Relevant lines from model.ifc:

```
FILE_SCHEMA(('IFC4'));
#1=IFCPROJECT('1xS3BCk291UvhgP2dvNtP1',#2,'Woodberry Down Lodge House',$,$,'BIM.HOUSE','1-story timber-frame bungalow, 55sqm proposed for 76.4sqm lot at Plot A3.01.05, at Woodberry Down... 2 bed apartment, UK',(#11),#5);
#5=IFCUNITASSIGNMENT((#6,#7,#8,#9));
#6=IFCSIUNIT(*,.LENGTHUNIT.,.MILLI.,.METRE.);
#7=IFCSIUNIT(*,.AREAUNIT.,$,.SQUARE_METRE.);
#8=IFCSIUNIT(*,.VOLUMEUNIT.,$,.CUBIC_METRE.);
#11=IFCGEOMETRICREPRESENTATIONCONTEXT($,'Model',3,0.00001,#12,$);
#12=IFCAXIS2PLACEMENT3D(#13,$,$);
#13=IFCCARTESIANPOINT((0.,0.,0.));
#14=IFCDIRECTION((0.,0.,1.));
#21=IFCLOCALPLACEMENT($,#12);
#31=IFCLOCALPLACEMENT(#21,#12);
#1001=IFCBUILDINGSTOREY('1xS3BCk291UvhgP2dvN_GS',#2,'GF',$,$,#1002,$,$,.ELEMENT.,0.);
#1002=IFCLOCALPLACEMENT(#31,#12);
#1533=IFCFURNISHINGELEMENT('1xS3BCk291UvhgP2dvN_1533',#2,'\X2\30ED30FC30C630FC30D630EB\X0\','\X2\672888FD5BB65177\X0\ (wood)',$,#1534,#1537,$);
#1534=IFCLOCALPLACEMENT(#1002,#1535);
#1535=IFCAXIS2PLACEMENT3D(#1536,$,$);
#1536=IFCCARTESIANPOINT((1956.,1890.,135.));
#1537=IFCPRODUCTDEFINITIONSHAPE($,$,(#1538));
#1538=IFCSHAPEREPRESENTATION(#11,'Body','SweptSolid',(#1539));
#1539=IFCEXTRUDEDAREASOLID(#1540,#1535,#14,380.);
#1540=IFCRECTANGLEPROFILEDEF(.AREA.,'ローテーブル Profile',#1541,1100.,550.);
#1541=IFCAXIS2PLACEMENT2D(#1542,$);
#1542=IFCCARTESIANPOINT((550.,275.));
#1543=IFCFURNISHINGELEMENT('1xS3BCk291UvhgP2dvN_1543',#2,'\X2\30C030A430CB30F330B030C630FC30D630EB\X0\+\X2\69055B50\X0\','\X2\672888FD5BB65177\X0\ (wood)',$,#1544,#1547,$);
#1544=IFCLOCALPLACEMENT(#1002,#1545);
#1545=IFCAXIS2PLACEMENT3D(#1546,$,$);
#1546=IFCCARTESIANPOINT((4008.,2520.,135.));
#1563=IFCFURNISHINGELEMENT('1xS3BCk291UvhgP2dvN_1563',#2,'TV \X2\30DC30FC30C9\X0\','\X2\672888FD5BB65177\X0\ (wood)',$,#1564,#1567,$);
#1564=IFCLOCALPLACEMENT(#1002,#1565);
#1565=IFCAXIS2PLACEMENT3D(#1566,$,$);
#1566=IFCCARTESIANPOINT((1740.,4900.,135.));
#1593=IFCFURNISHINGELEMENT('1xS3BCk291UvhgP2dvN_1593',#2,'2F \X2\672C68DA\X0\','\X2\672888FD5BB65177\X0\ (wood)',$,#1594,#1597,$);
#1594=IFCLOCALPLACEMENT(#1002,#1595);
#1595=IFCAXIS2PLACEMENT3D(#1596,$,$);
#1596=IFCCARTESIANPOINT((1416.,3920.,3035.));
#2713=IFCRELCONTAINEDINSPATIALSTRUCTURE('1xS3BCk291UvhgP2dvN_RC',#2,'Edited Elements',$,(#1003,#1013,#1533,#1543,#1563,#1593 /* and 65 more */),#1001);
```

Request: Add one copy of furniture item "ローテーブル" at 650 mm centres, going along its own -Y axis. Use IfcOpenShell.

```python
import ifcopenshell
import ifcopenshell.api.geometry
import ifcopenshell.api.root
import ifcopenshell.util.element
import ifcopenshell.util.placement

model = ifcopenshell.open("model.ifc")


def reuse_history(source, copy):
    """copy_class also copies each property set's owner history, people and application; keep the originals."""
    for rel in copy.IsDefinedBy:
        if rel.is_a("IfcRelDefinesByProperties") and (history := rel.RelatingPropertyDefinition.OwnerHistory):
            rel.RelatingPropertyDefinition.OwnerHistory = source.OwnerHistory
            ifcopenshell.util.element.remove_deep2(model, history)


source = model.by_id(1533)
base = ifcopenshell.util.placement.get_local_placement(source.ObjectPlacement)
step = -base[:3, 1] * 650.0

for i in range(1, 2):
    copy = ifcopenshell.api.root.copy_class(model, product=source)
    copy.Representation = ifcopenshell.util.element.copy_deep(
        model, source.Representation, exclude=["IfcGeometricRepresentationContext", "IfcRepresentationMap"]
    )
    reuse_history(source, copy)
    matrix = base.copy()
    matrix[:3, 3] += i * step
    print("added at", matrix[:3, 3].round(3) + 0.0)
    ifcopenshell.api.geometry.edit_object_placement(model, product=copy, matrix=matrix, is_si=False)

model.write("model_updated.ifc")
```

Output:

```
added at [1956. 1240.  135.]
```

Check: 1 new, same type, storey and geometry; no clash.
